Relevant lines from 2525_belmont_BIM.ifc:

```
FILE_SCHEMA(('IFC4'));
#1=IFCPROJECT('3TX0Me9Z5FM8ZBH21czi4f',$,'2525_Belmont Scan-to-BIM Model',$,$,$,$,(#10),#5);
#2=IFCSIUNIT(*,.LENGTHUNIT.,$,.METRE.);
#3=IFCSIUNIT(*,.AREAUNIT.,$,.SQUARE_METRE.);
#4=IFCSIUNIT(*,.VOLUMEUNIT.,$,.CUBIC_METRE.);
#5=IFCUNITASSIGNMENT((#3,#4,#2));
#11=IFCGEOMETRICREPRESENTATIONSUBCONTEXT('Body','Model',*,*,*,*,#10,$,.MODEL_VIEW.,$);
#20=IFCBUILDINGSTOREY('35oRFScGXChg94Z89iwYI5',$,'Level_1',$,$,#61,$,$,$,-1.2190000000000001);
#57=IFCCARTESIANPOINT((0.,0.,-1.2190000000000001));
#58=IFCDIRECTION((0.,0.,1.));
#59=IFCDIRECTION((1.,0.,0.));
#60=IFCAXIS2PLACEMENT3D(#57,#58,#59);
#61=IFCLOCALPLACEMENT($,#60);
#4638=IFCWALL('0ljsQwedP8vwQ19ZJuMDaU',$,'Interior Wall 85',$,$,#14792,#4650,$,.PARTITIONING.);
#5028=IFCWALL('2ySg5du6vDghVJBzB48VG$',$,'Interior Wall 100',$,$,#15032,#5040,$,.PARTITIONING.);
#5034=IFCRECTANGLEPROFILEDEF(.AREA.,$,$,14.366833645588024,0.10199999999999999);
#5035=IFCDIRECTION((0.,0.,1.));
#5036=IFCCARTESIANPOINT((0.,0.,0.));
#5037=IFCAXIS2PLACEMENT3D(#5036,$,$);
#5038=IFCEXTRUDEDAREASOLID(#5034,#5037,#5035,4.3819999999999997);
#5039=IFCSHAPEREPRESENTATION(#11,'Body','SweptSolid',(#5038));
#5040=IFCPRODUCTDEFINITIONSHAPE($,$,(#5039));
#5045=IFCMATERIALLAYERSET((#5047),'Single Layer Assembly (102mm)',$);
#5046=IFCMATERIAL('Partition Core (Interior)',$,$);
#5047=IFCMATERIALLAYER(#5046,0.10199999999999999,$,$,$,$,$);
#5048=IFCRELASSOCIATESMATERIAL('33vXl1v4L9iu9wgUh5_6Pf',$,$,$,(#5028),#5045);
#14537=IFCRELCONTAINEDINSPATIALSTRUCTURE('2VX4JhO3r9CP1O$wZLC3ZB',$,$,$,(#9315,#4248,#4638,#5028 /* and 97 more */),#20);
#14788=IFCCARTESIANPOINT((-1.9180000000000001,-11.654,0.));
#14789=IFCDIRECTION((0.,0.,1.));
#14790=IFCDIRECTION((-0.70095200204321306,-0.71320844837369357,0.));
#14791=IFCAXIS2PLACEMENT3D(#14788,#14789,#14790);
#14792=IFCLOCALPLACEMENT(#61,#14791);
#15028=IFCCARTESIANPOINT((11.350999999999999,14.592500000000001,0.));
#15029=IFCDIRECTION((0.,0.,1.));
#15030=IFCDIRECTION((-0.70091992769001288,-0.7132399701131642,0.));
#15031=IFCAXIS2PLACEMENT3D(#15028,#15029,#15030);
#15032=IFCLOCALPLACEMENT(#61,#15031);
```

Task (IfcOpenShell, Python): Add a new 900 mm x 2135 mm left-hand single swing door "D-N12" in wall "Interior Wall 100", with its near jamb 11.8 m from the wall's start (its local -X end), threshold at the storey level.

```python
import numpy as np
import ifcopenshell
import ifcopenshell.api.feature
import ifcopenshell.api.geometry
import ifcopenshell.api.root
import ifcopenshell.api.spatial
import ifcopenshell.geom
import ifcopenshell.util.element
import ifcopenshell.util.placement
import ifcopenshell.util.representation
import ifcopenshell.util.shape
import ifcopenshell.util.unit

model = ifcopenshell.open("2525_belmont_BIM.ifc")
unit_scale = ifcopenshell.util.unit.calculate_unit_scale(model)
settings = ifcopenshell.geom.settings()


def volume(element):
    """Net volume in cubic metres, openings subtracted."""
    shape = ifcopenshell.geom.create_shape(settings, element)
    return ifcopenshell.util.shape.get_volume(shape.geometry)


wall = model.by_guid("2ySg5du6vDghVJBzB48VG$")
storey = ifcopenshell.util.element.get_container(wall, ifc_class="IfcBuildingStorey")
context = ifcopenshell.util.representation.get_context(model, "Model", "Body", "MODEL_VIEW")
before = volume(wall)

width, height, from_end, sill = 0.9, 2.135, 11.8, 0.0  # metres

# The wall runs along its own X axis, and the end named is its -X end.
wall_shape = ifcopenshell.geom.create_shape(settings, wall)
x, y, z = ifcopenshell.util.shape.get_vertices(wall_shape.geometry).T
start = x.min() + from_end
face, thickness = float(y.min()), float(y.max() - y.min())
wall_matrix = ifcopenshell.util.placement.get_local_placement(wall.ObjectPlacement)
level = ifcopenshell.util.placement.get_local_placement(storey.ObjectPlacement)[2, 3]


def in_wall(x, y):
    """Placement at x, y metres in the wall's axes, at sill height."""
    matrix = wall_matrix.copy()
    matrix[:, 3] = wall_matrix @ np.array([x / unit_scale, y / unit_scale, 0.0, 1.0])
    matrix[2, 3] = level + sill / unit_scale
    return matrix


# Opening: a box that overshoots both wall faces by 50 mm.
opening = ifcopenshell.api.root.create_entity(model, ifc_class="IfcOpeningElement", predefined_type="OPENING")
box = ifcopenshell.api.geometry.add_wall_representation(
    model, context=context, length=width, height=height, thickness=thickness + 0.1
)
ifcopenshell.api.geometry.assign_representation(model, product=opening, representation=box)
ifcopenshell.api.geometry.edit_object_placement(model, product=opening, matrix=in_wall(start, face - 0.05), is_si=False)
ifcopenshell.api.feature.add_feature(model, feature=opening, element=wall)

door = ifcopenshell.api.root.create_entity(model, ifc_class="IfcDoor", name="D-N12", predefined_type="DOOR")
door.OverallWidth, door.OverallHeight = width / unit_scale, height / unit_scale
door.OperationType = "SINGLE_SWING_LEFT"
body = ifcopenshell.api.geometry.add_door_representation(
    model,
    context=context,
    overall_width=door.OverallWidth,
    overall_height=door.OverallHeight,
    operation_type="SINGLE_SWING_LEFT",
    lining_properties={"LiningDepth": thickness / unit_scale, "ThresholdDepth": thickness / unit_scale},
)
ifcopenshell.api.geometry.assign_representation(model, product=door, representation=body)
ifcopenshell.api.spatial.assign_container(model, products=[door], relating_structure=storey)
ifcopenshell.api.feature.add_filling(model, opening=opening, element=door)

# The lining spans the wall, so the door starts at the wall face.
ifcopenshell.api.geometry.edit_object_placement(model, product=door, matrix=in_wall(start, face), is_si=False)

after = volume(wall)

print(f"wall volume {before:.3f} -> {after:.3f} m3")

model.write("2525_belmont_BIM_rev.ifc")
```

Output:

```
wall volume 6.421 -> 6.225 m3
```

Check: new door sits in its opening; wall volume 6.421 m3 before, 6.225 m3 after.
